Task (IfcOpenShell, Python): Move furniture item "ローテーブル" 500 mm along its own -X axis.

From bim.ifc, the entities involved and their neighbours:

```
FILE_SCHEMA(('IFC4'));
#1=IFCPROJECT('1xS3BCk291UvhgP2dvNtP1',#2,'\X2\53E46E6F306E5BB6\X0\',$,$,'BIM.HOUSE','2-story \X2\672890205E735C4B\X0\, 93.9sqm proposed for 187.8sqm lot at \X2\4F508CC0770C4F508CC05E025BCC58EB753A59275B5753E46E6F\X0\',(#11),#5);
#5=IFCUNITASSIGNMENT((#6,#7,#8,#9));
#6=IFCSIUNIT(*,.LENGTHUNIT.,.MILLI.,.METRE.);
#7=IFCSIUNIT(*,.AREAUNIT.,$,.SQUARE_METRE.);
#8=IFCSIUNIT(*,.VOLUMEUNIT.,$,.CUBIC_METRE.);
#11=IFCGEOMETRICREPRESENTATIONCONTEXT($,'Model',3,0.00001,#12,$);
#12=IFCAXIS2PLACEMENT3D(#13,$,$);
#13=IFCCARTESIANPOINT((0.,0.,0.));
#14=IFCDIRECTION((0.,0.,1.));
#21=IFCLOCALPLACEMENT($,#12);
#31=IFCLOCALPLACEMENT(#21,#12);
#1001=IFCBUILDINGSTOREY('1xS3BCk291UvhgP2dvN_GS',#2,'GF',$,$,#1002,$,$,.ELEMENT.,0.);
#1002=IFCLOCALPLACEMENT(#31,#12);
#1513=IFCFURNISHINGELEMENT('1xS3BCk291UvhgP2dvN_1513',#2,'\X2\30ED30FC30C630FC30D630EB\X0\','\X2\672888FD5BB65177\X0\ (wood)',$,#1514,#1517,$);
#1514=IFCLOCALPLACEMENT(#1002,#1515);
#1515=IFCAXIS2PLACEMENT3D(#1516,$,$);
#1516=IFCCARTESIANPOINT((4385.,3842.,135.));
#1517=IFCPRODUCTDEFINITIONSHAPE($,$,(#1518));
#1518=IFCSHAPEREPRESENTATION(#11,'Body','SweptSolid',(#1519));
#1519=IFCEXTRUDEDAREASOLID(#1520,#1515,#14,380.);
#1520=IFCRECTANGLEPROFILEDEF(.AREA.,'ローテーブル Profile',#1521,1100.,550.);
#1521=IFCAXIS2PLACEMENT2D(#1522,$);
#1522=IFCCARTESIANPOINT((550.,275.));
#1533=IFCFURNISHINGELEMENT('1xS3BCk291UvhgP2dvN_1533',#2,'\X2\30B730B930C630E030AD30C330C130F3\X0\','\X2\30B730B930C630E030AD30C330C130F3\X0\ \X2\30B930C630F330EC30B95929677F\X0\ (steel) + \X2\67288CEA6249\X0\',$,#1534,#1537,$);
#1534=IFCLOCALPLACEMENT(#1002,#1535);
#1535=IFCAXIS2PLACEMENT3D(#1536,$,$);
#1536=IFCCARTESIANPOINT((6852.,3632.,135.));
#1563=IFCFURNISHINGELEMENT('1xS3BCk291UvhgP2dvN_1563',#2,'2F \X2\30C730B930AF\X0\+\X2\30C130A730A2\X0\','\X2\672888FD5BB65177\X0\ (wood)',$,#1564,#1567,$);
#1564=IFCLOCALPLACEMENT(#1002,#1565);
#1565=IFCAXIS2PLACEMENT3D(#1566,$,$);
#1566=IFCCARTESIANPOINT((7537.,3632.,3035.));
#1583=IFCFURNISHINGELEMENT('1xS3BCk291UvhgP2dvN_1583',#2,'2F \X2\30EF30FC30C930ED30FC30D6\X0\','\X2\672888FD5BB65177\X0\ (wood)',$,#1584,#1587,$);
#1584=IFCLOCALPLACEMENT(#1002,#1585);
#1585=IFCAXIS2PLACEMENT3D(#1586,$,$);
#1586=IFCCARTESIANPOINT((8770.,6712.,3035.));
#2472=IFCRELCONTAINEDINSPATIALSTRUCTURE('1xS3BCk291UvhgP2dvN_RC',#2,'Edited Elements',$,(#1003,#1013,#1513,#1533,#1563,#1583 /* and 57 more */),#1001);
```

```python
import ifcopenshell
import ifcopenshell.api.geometry
import ifcopenshell.util.placement
import ifcopenshell.util.unit

model = ifcopenshell.open("bim.ifc")
unit_scale = ifcopenshell.util.unit.calculate_unit_scale(model)

item = model.by_guid("1xS3BCk291UvhgP2dvN_1513")
matrix = ifcopenshell.util.placement.get_local_placement(item.ObjectPlacement)
matrix[:3, 3] -= matrix[:3, 0] * 0.5 / unit_scale
ifcopenshell.api.geometry.edit_object_placement(model, product=item, matrix=matrix, is_si=False)

print(ifcopenshell.util.placement.get_local_placement(item.ObjectPlacement).round(3) + 0.0)

model.write("bim_rev.ifc")
```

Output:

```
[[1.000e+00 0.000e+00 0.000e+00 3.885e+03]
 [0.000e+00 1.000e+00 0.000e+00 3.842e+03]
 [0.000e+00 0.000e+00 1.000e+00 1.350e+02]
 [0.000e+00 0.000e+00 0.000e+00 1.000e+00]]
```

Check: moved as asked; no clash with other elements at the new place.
